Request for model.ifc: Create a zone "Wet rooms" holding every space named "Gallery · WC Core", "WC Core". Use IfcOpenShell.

First a look at what the model holds.

```python
import ifcopenshell

model = ifcopenshell.open("model.ifc")
print(model.schema)
seen = {}
for space in model.by_type("IfcSpace"):
    seen[space.Name] = seen.get(space.Name, 0) + 1
for name, count in sorted(seen.items(), key=str):
    print(count, "x", name)
print("zones:", [z.Name for z in model.by_type("IfcZone")][:20])
```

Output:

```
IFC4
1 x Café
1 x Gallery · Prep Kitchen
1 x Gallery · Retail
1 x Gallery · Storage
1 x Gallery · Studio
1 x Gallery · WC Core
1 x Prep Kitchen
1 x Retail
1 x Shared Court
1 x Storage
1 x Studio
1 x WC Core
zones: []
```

```python
import ifcopenshell
import ifcopenshell.api.group
import ifcopenshell.api.root

model = ifcopenshell.open("model.ifc")

names = {"Gallery · WC Core", "WC Core"}
spaces = [s for s in model.by_type("IfcSpace") if s.Name in names]

zone = ifcopenshell.api.root.create_entity(model, ifc_class="IfcZone", name="Wet rooms")
ifcopenshell.api.group.assign_group(model, products=spaces, group=zone)
print(len(spaces), "spaces in", zone.Name)

model.write("model_updated.ifc")
```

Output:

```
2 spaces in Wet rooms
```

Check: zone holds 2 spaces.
